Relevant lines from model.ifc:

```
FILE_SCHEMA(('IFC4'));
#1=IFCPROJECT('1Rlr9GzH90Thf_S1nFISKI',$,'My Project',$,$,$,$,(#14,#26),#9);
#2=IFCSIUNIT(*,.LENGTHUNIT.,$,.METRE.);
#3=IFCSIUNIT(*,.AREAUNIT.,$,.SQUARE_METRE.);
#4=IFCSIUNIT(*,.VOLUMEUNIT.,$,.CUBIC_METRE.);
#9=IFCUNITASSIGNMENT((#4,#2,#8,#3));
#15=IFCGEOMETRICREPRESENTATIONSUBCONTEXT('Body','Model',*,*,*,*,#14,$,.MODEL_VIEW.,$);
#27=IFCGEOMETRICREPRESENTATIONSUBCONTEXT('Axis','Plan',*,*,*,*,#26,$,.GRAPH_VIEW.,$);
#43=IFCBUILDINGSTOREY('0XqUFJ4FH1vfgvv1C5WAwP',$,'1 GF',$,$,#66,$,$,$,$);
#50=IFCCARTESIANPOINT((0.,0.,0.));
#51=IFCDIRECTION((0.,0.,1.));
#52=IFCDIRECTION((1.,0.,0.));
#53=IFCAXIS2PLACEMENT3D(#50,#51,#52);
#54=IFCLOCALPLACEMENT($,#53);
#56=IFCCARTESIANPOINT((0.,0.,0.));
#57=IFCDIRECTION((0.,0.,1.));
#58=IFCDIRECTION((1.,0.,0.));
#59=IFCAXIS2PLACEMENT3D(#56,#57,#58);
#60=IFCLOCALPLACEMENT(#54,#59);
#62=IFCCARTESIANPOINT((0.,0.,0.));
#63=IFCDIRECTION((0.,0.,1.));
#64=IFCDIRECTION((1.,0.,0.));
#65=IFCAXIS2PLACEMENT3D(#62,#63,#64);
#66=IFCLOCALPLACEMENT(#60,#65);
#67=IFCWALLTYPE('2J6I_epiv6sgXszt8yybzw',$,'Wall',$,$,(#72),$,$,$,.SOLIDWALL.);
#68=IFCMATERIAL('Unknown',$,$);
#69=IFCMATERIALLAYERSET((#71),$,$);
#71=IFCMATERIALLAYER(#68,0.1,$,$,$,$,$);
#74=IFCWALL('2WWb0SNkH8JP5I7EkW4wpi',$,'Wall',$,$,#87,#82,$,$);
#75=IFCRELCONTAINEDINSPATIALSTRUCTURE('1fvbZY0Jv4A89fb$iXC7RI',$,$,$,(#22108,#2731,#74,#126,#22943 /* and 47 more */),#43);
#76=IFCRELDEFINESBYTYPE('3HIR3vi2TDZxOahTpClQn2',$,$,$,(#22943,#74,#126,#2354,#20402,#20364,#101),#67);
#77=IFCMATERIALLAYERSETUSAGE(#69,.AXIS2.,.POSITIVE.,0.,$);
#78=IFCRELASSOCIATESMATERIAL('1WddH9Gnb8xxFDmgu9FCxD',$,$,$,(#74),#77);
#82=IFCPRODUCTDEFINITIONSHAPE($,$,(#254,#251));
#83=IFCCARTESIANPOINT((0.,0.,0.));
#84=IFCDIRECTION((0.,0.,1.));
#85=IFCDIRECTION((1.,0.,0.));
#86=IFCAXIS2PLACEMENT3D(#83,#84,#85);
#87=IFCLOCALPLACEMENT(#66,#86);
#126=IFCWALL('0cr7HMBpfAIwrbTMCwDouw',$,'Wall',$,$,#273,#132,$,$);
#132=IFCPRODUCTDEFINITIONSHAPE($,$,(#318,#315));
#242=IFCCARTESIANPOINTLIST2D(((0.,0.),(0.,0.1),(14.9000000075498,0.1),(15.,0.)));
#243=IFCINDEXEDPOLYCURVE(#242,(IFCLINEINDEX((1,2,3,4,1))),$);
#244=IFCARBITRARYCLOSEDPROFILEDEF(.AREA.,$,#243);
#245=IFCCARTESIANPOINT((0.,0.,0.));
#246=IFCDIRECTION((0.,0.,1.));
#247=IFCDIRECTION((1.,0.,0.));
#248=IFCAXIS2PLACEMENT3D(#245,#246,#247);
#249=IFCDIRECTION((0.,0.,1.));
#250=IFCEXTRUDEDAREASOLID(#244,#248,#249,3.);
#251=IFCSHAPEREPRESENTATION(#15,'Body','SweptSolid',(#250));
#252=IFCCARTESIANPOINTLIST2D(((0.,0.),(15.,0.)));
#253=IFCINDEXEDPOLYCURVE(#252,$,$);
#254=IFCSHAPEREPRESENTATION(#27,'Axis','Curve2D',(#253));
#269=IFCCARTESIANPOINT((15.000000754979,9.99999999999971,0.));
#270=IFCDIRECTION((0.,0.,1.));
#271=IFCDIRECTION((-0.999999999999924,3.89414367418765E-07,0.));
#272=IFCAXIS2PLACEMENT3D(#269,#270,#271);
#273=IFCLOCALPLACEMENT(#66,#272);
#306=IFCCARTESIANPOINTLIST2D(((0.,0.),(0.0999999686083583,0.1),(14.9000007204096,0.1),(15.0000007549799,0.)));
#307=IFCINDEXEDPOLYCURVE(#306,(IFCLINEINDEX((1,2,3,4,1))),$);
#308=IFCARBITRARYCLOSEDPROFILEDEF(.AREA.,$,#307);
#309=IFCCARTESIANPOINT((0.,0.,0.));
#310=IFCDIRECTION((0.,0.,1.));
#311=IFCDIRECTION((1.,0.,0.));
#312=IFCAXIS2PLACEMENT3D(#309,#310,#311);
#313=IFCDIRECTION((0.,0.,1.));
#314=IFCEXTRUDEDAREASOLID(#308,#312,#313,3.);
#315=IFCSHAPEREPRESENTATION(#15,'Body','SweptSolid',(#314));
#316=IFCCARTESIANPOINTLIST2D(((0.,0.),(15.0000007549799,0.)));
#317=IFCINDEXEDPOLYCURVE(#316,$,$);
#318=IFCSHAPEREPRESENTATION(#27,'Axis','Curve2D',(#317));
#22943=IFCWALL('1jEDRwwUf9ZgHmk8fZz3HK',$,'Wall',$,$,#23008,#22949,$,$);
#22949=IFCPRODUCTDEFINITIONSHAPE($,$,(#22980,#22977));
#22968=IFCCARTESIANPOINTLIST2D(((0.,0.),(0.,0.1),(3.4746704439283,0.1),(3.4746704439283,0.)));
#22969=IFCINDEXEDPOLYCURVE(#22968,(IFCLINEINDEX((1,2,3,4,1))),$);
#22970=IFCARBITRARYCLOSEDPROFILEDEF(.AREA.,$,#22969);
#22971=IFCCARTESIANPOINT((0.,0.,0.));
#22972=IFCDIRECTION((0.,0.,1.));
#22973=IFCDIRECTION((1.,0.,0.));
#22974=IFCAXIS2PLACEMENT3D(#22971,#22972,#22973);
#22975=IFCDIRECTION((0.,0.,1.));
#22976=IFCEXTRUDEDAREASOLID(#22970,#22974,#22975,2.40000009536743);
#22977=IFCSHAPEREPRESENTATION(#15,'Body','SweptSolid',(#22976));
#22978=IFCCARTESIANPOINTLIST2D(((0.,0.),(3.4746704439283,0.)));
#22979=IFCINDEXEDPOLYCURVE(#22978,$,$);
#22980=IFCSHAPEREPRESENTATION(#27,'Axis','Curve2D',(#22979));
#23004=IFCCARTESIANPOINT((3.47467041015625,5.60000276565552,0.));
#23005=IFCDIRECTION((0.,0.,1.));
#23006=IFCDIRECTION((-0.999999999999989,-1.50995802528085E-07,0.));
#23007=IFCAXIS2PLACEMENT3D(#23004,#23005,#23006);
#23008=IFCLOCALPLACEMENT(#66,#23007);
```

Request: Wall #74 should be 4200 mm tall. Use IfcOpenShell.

```python
import ifcopenshell
import ifcopenshell.geom
import ifcopenshell.util.representation
import ifcopenshell.util.shape
import ifcopenshell.util.unit

model = ifcopenshell.open("model.ifc")
unit_scale = ifcopenshell.util.unit.calculate_unit_scale(model)
settings = ifcopenshell.geom.settings()


def volume(element):
    """Net volume in cubic metres, openings subtracted."""
    shape = ifcopenshell.geom.create_shape(settings, element)
    return ifcopenshell.util.shape.get_volume(shape.geometry)


wall = model.by_guid("2WWb0SNkH8JP5I7EkW4wpi")
before = volume(wall)

body = ifcopenshell.util.representation.get_representation(wall, "Model", "Body")
solid = body.Items[0]
old_height = solid.Depth
solid.Depth = 4.2 / unit_scale
after = volume(wall)

print(f"height {old_height:g} -> {solid.Depth:g}, volume {before:.3f} -> {after:.3f} m3")

model.write("model_v2.ifc")
```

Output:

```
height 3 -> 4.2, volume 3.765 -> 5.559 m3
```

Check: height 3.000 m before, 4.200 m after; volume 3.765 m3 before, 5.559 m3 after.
